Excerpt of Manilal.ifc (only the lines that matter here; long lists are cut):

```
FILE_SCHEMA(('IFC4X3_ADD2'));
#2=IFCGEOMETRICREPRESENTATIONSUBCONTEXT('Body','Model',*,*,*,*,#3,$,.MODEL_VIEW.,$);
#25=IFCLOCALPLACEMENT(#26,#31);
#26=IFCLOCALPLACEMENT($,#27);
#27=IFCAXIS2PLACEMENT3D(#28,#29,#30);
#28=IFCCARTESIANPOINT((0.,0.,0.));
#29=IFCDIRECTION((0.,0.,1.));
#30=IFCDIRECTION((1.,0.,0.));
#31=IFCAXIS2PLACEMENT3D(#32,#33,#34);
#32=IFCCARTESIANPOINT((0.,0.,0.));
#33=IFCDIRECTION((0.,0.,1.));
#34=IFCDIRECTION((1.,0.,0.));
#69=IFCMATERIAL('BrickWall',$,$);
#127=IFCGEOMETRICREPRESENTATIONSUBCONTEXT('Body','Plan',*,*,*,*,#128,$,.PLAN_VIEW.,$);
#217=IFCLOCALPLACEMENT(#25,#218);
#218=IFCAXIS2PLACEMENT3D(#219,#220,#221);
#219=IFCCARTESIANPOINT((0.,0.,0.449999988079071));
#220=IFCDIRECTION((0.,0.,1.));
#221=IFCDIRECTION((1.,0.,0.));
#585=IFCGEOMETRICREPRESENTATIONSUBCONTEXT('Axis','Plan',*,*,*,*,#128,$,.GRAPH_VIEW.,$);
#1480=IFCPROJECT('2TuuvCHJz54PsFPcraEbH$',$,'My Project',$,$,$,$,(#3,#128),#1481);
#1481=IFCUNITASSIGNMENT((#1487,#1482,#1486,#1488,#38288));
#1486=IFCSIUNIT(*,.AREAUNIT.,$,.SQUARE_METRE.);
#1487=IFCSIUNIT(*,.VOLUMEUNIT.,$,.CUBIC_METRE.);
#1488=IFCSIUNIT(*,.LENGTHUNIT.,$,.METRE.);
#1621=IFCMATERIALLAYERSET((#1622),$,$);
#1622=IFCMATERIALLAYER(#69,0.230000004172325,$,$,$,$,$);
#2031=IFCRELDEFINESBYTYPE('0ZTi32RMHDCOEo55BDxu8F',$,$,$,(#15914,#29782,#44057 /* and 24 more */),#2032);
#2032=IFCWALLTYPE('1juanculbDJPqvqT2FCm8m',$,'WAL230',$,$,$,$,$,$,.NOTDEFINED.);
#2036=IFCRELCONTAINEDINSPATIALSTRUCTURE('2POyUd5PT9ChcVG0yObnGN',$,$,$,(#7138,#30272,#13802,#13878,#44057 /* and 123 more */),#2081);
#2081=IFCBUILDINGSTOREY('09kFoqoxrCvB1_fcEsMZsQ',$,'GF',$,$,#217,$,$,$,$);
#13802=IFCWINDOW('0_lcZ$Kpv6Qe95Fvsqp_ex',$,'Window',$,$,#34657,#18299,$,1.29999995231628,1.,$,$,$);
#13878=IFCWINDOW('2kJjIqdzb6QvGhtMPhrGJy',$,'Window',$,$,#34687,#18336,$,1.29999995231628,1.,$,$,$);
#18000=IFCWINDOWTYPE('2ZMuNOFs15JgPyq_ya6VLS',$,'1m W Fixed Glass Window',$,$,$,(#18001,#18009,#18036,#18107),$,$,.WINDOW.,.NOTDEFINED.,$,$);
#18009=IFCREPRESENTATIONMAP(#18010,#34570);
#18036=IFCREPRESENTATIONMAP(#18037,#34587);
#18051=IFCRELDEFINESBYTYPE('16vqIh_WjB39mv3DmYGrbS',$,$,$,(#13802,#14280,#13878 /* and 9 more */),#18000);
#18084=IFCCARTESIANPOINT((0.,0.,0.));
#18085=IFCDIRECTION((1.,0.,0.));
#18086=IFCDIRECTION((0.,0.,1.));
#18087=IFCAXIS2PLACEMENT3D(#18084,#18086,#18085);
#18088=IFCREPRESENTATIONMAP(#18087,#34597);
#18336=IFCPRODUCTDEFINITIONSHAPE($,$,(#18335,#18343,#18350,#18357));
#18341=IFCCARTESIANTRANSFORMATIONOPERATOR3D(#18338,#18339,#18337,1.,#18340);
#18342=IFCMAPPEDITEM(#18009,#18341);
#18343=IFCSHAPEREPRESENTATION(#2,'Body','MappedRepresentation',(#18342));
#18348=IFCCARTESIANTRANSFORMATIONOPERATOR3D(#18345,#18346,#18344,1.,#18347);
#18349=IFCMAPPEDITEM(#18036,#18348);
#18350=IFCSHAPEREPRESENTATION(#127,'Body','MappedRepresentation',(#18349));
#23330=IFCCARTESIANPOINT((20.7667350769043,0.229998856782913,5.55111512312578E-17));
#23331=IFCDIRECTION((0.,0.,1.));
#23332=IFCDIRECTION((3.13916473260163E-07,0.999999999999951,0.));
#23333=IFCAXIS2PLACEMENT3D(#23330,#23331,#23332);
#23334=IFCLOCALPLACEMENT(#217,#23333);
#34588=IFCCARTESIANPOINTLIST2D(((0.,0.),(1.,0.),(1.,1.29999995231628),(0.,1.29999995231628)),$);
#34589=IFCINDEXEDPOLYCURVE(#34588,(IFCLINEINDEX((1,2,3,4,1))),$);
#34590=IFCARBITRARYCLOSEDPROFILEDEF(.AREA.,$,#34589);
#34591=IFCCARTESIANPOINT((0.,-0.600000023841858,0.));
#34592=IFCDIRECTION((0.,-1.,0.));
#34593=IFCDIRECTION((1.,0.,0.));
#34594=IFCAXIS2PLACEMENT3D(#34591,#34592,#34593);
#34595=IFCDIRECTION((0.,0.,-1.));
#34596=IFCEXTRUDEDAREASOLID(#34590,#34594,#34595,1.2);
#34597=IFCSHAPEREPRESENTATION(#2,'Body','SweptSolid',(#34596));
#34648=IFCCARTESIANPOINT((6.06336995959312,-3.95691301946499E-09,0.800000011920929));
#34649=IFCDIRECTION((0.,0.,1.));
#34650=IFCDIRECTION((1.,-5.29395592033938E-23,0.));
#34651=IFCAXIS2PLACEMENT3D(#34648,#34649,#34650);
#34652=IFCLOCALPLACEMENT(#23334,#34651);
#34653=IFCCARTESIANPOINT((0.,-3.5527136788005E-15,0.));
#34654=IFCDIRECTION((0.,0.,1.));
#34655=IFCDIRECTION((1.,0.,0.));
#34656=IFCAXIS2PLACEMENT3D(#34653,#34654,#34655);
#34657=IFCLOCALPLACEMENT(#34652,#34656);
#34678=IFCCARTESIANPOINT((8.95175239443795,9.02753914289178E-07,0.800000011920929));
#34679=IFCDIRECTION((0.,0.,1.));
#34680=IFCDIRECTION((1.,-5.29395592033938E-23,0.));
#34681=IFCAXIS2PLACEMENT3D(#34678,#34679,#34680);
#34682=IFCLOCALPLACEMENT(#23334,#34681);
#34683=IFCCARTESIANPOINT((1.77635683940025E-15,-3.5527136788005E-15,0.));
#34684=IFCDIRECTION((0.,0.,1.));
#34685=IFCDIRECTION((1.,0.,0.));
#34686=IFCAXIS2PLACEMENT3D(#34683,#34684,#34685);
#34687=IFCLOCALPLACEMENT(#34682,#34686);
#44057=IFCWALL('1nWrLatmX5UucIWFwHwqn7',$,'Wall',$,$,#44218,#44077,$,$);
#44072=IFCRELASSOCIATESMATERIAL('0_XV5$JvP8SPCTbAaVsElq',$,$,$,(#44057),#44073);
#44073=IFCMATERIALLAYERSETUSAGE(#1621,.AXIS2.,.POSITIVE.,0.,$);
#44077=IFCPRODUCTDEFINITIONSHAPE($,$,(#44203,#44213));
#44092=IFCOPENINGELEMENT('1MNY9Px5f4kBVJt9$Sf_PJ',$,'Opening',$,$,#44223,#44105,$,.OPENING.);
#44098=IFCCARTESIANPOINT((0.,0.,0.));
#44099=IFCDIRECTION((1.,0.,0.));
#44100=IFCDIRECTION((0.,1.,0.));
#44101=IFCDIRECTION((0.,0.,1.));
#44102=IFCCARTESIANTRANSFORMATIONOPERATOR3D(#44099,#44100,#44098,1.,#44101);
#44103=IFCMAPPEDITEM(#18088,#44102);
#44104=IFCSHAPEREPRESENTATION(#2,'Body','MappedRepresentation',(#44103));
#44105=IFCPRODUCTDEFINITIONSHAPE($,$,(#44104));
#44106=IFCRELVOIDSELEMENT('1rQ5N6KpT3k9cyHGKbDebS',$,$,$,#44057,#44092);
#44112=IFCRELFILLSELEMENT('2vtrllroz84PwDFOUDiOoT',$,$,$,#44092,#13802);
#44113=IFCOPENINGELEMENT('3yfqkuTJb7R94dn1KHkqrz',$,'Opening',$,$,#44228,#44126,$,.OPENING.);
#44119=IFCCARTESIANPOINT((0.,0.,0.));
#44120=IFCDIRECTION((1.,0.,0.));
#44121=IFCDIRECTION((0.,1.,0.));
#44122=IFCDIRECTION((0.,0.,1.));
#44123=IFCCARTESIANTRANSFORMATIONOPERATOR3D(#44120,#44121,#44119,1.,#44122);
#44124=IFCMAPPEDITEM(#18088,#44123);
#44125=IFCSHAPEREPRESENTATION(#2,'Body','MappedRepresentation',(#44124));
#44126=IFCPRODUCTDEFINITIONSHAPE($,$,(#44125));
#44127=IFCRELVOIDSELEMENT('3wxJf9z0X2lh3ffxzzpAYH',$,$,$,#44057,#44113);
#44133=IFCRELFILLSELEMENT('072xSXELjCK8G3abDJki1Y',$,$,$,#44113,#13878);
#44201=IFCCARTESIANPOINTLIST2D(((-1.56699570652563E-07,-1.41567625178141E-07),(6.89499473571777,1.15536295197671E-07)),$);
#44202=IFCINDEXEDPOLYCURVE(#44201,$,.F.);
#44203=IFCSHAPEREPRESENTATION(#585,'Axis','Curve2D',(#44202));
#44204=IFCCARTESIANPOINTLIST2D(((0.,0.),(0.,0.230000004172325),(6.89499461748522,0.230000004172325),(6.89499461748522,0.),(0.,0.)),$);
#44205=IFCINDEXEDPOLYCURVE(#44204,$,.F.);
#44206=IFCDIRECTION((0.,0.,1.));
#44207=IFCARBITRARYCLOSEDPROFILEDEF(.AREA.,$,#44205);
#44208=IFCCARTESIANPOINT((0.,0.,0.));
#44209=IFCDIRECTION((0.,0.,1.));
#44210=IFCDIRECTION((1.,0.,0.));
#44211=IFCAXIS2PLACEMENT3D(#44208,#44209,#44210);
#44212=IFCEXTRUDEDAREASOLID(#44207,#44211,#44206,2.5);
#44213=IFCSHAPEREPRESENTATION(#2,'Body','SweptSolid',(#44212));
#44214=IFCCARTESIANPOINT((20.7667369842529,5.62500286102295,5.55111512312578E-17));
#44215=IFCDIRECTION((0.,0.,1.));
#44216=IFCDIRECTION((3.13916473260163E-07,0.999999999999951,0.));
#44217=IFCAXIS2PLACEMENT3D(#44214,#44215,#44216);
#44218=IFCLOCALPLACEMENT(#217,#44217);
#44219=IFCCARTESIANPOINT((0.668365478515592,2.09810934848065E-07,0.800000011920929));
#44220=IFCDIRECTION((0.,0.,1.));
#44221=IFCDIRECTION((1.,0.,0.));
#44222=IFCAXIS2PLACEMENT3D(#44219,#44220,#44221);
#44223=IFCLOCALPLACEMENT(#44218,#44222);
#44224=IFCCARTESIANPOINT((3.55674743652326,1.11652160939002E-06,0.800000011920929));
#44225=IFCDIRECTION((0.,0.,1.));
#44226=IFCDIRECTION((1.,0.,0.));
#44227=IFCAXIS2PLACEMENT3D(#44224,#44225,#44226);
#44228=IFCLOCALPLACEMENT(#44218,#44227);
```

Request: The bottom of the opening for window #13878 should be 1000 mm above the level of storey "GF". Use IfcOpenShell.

```python
import numpy as np
import ifcopenshell
import ifcopenshell.api.geometry
import ifcopenshell.geom
import ifcopenshell.util.element
import ifcopenshell.util.placement
import ifcopenshell.util.shape
import ifcopenshell.util.unit

model = ifcopenshell.open("Manilal.ifc")
unit_scale = ifcopenshell.util.unit.calculate_unit_scale(model)

window = model.by_guid("2kJjIqdzb6QvGhtMPhrGJy")
opening = window.FillsVoids[0].RelatingOpeningElement
storey = ifcopenshell.util.element.get_container(window, ifc_class="IfcBuildingStorey")
level = ifcopenshell.util.placement.get_local_placement(storey.ObjectPlacement)[2, 3]

# The opening's origin need not be at the sill, so measure its lowest point.
shape = ifcopenshell.geom.create_shape(ifcopenshell.geom.settings(), opening)
bottom = ifcopenshell.util.shape.get_shape_bottom_elevation(shape, shape.geometry) / unit_scale
dz = level + 1 / unit_scale - bottom

shift = np.array([0.0, 0.0, dz])
# The window is not placed relative to its opening, so move both.
for product in (opening, window):
    matrix = ifcopenshell.util.placement.get_local_placement(product.ObjectPlacement)
    matrix[:3, 3] += shift
    ifcopenshell.api.geometry.edit_object_placement(model, product=product, matrix=matrix, is_si=False)

print(f"moved by {dz * unit_scale:+.3f} m")

model.write("Manilal-out.ifc")
```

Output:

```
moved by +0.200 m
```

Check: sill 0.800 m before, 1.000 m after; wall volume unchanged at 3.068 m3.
